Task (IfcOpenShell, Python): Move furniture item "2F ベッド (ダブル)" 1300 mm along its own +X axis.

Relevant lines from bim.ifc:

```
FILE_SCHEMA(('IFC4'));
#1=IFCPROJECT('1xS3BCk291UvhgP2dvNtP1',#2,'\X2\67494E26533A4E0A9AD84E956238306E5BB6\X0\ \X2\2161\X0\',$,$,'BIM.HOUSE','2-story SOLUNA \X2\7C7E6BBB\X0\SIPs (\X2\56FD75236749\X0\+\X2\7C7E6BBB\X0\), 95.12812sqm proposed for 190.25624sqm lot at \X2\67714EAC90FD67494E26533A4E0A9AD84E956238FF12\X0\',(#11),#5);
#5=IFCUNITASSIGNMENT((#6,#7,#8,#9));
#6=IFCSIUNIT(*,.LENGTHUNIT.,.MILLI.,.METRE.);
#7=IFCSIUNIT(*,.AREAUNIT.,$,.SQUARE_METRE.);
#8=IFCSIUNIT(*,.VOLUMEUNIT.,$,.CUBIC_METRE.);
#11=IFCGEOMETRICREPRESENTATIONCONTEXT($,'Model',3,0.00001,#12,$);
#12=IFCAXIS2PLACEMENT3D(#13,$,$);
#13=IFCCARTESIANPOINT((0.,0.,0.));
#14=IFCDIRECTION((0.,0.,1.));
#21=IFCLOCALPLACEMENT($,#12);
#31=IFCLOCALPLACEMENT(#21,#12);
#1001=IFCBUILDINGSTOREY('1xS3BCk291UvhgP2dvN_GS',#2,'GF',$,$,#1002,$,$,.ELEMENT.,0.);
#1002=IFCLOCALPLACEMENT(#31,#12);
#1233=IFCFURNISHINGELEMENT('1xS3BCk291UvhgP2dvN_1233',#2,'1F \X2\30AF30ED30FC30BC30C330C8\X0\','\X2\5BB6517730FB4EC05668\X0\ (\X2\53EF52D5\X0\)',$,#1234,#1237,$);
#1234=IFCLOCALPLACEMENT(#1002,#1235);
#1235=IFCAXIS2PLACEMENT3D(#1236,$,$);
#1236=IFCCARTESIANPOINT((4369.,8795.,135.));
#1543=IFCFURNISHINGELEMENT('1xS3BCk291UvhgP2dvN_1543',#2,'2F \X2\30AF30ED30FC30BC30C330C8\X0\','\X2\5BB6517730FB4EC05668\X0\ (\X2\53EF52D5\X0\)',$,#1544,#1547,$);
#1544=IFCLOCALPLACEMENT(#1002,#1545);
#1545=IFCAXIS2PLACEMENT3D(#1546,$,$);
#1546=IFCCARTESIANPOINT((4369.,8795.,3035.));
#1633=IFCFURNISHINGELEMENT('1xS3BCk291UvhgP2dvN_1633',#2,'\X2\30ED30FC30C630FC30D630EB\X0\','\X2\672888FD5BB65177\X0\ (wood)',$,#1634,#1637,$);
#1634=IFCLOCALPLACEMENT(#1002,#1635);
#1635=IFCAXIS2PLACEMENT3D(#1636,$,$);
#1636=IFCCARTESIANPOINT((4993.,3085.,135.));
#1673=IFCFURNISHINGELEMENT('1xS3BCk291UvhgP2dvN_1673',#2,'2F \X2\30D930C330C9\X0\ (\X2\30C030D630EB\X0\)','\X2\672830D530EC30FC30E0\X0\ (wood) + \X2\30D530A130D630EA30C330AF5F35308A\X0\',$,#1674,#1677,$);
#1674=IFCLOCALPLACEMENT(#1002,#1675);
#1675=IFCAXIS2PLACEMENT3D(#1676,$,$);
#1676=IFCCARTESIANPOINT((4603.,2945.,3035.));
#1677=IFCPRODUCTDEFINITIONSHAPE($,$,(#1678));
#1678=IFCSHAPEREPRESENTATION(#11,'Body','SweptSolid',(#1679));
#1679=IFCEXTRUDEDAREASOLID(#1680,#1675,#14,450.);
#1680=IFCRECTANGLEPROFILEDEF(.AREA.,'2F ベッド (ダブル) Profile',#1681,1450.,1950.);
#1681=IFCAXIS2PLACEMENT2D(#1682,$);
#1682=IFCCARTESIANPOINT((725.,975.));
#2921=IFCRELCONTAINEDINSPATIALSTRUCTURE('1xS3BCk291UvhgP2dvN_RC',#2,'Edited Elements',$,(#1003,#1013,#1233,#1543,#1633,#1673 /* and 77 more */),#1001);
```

```python
import ifcopenshell
import ifcopenshell.api.geometry
import ifcopenshell.util.placement
import ifcopenshell.util.unit

model = ifcopenshell.open("bim.ifc")
unit_scale = ifcopenshell.util.unit.calculate_unit_scale(model)

item = model.by_guid("1xS3BCk291UvhgP2dvN_1673")
matrix = ifcopenshell.util.placement.get_local_placement(item.ObjectPlacement)
matrix[:3, 3] += matrix[:3, 0] * 1.3 / unit_scale
ifcopenshell.api.geometry.edit_object_placement(model, product=item, matrix=matrix, is_si=False)

print(ifcopenshell.util.placement.get_local_placement(item.ObjectPlacement).round(3) + 0.0)

model.write("bim_updated.ifc")
```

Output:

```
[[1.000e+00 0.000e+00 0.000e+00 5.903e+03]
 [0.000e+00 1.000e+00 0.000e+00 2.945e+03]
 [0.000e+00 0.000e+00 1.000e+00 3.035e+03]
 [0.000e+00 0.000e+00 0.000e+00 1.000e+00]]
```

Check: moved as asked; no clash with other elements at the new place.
